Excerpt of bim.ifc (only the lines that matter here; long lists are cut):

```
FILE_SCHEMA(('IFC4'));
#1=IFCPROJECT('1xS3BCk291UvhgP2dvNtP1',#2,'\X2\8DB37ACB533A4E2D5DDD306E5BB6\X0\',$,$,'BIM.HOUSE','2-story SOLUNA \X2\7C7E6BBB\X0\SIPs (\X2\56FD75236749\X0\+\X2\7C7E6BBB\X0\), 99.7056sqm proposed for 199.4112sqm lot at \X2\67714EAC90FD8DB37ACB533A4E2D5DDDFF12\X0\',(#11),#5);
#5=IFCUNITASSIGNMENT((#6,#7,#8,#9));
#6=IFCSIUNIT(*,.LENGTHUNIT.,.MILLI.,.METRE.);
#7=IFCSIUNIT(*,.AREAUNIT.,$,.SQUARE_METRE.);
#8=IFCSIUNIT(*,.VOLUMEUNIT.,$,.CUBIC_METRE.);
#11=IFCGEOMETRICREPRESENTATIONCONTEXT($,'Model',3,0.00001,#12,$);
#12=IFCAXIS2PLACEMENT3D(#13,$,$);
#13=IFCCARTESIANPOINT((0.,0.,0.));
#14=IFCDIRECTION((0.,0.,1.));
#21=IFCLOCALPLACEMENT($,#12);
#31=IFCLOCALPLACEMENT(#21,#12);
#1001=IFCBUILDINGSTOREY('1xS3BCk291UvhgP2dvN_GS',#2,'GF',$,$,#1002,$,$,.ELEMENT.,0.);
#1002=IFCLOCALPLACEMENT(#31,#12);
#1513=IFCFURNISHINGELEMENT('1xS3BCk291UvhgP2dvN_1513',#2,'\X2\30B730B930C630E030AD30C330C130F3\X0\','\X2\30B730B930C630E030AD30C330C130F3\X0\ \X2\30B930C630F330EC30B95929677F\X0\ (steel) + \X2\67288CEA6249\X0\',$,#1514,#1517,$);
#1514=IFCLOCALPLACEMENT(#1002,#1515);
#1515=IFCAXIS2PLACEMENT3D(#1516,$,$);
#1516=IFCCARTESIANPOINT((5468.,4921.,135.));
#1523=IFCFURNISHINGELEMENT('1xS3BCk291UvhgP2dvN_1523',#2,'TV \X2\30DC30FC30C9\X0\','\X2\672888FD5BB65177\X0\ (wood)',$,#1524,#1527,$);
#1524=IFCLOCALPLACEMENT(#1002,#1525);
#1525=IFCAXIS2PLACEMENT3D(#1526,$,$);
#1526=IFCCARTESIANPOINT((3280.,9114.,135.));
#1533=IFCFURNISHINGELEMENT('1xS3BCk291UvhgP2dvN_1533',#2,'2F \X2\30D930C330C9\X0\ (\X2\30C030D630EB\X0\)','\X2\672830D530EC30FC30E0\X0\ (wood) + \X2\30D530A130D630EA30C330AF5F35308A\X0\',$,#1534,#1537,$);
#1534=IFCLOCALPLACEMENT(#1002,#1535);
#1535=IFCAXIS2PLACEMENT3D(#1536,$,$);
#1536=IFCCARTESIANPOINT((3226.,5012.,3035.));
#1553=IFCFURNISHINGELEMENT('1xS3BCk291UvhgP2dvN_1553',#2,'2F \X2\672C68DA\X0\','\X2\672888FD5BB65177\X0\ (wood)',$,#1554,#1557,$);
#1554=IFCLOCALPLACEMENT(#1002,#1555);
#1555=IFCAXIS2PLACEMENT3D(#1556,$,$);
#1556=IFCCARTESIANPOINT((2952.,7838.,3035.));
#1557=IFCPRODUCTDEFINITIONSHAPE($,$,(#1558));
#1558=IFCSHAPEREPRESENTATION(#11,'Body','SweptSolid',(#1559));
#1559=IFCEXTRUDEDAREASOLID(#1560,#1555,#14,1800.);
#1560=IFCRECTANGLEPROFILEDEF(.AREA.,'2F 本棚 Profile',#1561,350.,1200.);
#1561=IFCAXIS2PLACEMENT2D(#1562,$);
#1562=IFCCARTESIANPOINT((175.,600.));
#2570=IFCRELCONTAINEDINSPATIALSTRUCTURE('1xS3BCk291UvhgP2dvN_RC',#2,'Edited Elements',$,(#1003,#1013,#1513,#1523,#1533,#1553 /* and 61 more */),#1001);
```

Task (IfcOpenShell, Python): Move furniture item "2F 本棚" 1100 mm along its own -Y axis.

```python
import ifcopenshell
import ifcopenshell.api.geometry
import ifcopenshell.util.placement
import ifcopenshell.util.unit

model = ifcopenshell.open("bim.ifc")
unit_scale = ifcopenshell.util.unit.calculate_unit_scale(model)

item = model.by_guid("1xS3BCk291UvhgP2dvN_1553")
matrix = ifcopenshell.util.placement.get_local_placement(item.ObjectPlacement)
matrix[:3, 3] -= matrix[:3, 1] * 1.1 / unit_scale
ifcopenshell.api.geometry.edit_object_placement(model, product=item, matrix=matrix, is_si=False)

print(ifcopenshell.util.placement.get_local_placement(item.ObjectPlacement).round(3) + 0.0)

model.write("bim_edited.ifc")
```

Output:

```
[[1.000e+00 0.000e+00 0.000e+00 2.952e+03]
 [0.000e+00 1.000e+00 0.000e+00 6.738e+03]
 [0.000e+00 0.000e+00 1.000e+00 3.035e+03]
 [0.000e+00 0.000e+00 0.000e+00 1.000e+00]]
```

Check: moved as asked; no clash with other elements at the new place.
